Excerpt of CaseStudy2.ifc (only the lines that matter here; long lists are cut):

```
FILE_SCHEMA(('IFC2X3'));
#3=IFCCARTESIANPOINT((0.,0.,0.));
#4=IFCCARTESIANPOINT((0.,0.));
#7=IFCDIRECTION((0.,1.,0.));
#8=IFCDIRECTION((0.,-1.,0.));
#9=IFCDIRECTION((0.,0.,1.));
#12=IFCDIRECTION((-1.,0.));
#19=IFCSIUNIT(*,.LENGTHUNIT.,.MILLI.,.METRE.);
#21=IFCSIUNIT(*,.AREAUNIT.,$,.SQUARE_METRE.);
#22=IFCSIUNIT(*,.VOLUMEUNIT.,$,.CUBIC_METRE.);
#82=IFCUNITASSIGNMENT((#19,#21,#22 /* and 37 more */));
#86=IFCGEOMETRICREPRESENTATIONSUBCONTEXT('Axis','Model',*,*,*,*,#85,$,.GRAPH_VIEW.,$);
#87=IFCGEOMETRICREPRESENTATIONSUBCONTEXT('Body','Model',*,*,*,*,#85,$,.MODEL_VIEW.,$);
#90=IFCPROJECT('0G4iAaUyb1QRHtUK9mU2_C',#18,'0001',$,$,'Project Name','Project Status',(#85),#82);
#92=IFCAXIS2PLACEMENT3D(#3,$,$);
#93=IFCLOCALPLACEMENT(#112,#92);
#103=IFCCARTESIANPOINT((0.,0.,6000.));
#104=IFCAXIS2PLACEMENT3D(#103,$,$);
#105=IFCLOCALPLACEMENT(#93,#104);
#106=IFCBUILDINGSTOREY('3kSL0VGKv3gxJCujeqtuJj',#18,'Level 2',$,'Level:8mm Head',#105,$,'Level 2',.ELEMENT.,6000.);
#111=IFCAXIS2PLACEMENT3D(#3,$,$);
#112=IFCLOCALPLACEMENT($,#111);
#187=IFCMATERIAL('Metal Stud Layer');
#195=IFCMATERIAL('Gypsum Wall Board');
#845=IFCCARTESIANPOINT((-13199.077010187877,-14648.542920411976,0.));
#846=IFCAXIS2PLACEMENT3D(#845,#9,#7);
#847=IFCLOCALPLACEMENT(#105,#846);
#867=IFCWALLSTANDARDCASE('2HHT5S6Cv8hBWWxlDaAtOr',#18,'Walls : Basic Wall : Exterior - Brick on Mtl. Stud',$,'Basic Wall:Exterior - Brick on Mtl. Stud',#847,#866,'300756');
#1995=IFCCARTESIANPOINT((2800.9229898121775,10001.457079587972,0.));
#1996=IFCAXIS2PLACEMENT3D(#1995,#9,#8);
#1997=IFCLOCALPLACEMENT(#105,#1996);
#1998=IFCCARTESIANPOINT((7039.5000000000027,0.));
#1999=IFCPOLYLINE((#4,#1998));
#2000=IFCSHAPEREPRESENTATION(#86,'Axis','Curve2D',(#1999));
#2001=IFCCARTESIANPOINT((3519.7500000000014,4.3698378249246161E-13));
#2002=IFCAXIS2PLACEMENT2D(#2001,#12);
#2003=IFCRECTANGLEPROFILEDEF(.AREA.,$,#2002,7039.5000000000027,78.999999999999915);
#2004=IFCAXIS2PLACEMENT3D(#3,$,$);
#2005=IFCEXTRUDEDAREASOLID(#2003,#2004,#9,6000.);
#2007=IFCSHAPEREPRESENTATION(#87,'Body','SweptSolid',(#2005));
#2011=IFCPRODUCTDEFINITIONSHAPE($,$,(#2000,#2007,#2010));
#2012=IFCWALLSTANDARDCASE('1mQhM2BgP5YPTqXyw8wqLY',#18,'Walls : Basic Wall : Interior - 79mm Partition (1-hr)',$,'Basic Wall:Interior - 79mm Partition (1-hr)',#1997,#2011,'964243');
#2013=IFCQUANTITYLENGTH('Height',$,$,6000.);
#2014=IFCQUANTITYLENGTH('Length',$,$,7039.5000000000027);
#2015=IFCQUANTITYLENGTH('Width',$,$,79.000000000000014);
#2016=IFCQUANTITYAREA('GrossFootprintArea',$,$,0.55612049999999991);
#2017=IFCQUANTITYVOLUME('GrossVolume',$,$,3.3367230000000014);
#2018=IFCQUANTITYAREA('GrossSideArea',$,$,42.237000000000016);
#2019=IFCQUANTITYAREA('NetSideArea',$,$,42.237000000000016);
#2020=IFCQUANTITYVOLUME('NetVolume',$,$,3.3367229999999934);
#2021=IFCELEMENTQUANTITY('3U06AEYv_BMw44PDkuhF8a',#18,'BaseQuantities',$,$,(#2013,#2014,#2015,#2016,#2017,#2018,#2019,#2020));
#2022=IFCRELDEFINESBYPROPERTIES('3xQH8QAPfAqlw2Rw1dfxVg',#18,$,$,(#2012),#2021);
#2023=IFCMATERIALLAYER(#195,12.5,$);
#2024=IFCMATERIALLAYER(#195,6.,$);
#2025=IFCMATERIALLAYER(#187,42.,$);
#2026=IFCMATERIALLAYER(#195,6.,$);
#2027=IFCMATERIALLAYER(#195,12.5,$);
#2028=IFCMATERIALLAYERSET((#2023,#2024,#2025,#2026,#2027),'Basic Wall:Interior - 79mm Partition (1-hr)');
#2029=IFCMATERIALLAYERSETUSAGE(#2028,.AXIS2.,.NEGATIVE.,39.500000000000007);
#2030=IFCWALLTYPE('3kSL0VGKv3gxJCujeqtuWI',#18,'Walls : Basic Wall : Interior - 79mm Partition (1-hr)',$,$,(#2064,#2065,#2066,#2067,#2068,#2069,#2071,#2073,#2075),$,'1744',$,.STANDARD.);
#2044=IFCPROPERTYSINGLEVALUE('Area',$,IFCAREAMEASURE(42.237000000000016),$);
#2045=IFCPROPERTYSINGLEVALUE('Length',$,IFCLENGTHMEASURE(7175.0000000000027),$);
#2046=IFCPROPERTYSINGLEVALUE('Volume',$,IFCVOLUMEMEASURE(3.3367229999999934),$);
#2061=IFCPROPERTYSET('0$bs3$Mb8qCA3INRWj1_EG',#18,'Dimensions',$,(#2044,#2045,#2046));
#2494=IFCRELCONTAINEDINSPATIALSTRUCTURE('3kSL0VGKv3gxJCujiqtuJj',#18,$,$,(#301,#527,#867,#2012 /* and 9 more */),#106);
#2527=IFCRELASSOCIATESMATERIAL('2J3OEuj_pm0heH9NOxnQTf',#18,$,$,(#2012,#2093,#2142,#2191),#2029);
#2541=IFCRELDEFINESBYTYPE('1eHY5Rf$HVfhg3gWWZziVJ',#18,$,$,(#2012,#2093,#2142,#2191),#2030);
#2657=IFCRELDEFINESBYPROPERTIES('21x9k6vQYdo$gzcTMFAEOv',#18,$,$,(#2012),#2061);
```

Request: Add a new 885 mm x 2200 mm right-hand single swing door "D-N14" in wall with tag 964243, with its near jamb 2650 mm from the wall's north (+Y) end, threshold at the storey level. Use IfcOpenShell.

```python
import numpy as np
import ifcopenshell
import ifcopenshell.api.feature
import ifcopenshell.api.geometry
import ifcopenshell.api.pset
import ifcopenshell.api.root
import ifcopenshell.api.spatial
import ifcopenshell.api.type
import ifcopenshell.geom
import ifcopenshell.util.element
import ifcopenshell.util.placement
import ifcopenshell.util.representation
import ifcopenshell.util.shape
import ifcopenshell.util.unit

model = ifcopenshell.open("CaseStudy2.ifc")
unit_scale = ifcopenshell.util.unit.calculate_unit_scale(model)
area_scale = ifcopenshell.util.unit.calculate_unit_scale(model, "AREAUNIT")
volume_scale = ifcopenshell.util.unit.calculate_unit_scale(model, "VOLUMEUNIT")
settings = ifcopenshell.geom.settings()


def volume(element):
    """Net volume in cubic metres, openings subtracted."""
    shape = ifcopenshell.geom.create_shape(settings, element)
    return ifcopenshell.util.shape.get_volume(shape.geometry)


wall = model.by_guid("1mQhM2BgP5YPTqXyw8wqLY")
storey = ifcopenshell.util.element.get_container(wall, ifc_class="IfcBuildingStorey")
context = ifcopenshell.util.representation.get_context(model, "Model", "Body", "MODEL_VIEW")
before = volume(wall)

width, height, from_end, sill = 0.885, 2.2, 2.65, 0.0  # metres

# The wall runs along its own X axis, and the end named is its -X end.
wall_shape = ifcopenshell.geom.create_shape(settings, wall)
x, y, z = ifcopenshell.util.shape.get_vertices(wall_shape.geometry).T
start = x.min() + from_end
face, thickness = float(y.min()), float(y.max() - y.min())
wall_matrix = ifcopenshell.util.placement.get_local_placement(wall.ObjectPlacement)
level = ifcopenshell.util.placement.get_local_placement(storey.ObjectPlacement)[2, 3]


def in_wall(x, y):
    """Placement at x, y metres in the wall's axes, at sill height."""
    matrix = wall_matrix.copy()
    matrix[:, 3] = wall_matrix @ np.array([x / unit_scale, y / unit_scale, 0.0, 1.0])
    matrix[2, 3] = level + sill / unit_scale
    return matrix


# Opening: a box that overshoots both wall faces by 50 mm.
opening = ifcopenshell.api.root.create_entity(model, ifc_class="IfcOpeningElement")
box = ifcopenshell.api.geometry.add_wall_representation(
    model, context=context, length=width, height=height, thickness=thickness + 0.1
)
ifcopenshell.api.geometry.assign_representation(model, product=opening, representation=box)
ifcopenshell.api.geometry.edit_object_placement(model, product=opening, matrix=in_wall(start, face - 0.05), is_si=False)
ifcopenshell.api.feature.add_feature(model, feature=opening, element=wall)

door = ifcopenshell.api.root.create_entity(model, ifc_class="IfcDoor", name="D-N14")
door.OverallWidth, door.OverallHeight = width / unit_scale, height / unit_scale
body = ifcopenshell.api.geometry.add_door_representation(
    model,
    context=context,
    overall_width=door.OverallWidth,
    overall_height=door.OverallHeight,
    operation_type="SINGLE_SWING_RIGHT",
    lining_properties={"LiningDepth": thickness / unit_scale, "ThresholdDepth": thickness / unit_scale},
)
ifcopenshell.api.geometry.assign_representation(model, product=door, representation=body)
ifcopenshell.api.spatial.assign_container(model, products=[door], relating_structure=storey)
fills = ifcopenshell.api.feature.add_filling(model, opening=opening, element=door)
fills.OwnerHistory = door.OwnerHistory  # required in IFC2X3

# IFC2X3 keeps the operation on the door style.
style = ifcopenshell.api.root.create_entity(model, ifc_class="IfcDoorStyle", name="D-N14")
style.OperationType, style.ConstructionType = "SINGLE_SWING_RIGHT", "NOTDEFINED"
style.ParameterTakesPrecedence = style.Sizeable = False
ifcopenshell.api.type.assign_type(model, related_objects=[door], relating_type=style)

# The lining spans the wall, so the door starts at the wall face.
ifcopenshell.api.geometry.edit_object_placement(model, product=door, matrix=in_wall(start, face), is_si=False)

after = volume(wall)

# Update the wall's stored quantities.
qto = model.by_id(ifcopenshell.util.element.get_pset(wall, "BaseQuantities", should_inherit=False)["id"])
ifcopenshell.api.pset.edit_qto(model, qto=qto, properties={
    "NetSideArea": after / thickness / area_scale,
    "NetVolume": after / volume_scale,
})
pset = model.by_id(ifcopenshell.util.element.get_pset(wall, "Dimensions", should_inherit=False)["id"])
ifcopenshell.api.pset.edit_pset(model, pset=pset, properties={
    "Area": model.create_entity("IfcAreaMeasure", after / thickness / area_scale),
    "Volume": model.create_entity("IfcVolumeMeasure", after / volume_scale),
})

print(f"wall volume {before:.3f} -> {after:.3f} m3")

model.write("CaseStudy2_rev.ifc")
```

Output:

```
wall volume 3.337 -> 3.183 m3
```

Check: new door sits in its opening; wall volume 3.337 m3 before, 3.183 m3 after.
